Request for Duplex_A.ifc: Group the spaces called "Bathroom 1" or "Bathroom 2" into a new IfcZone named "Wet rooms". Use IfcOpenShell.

First a look at what the model holds.

```python
import ifcopenshell

model = ifcopenshell.open("Duplex_A.ifc")
print(model.schema)
seen = {}
for space in model.by_type("IfcSpace"):
    seen[space.LongName] = seen.get(space.LongName, 0) + 1
for name, count in sorted(seen.items(), key=str):
    print(count, "x", name)
print("zones:", [z.Name for z in model.by_type("IfcZone")][:20])
```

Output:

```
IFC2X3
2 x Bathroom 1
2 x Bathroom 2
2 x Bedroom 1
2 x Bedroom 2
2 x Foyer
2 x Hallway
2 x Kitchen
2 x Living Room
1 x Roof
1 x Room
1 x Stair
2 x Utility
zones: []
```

```python
import ifcopenshell
import ifcopenshell.api.group
import ifcopenshell.api.root

model = ifcopenshell.open("Duplex_A.ifc")

names = {"Bathroom 1", "Bathroom 2"}
spaces = [s for s in model.by_type("IfcSpace") if s.LongName in names]

zone = ifcopenshell.api.root.create_entity(model, ifc_class="IfcZone", name="Wet rooms")
ifcopenshell.api.group.assign_group(model, products=spaces, group=zone)
print(len(spaces), "spaces in", zone.Name)

model.write("Duplex_A_edited.ifc")
```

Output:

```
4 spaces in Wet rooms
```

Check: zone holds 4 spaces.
